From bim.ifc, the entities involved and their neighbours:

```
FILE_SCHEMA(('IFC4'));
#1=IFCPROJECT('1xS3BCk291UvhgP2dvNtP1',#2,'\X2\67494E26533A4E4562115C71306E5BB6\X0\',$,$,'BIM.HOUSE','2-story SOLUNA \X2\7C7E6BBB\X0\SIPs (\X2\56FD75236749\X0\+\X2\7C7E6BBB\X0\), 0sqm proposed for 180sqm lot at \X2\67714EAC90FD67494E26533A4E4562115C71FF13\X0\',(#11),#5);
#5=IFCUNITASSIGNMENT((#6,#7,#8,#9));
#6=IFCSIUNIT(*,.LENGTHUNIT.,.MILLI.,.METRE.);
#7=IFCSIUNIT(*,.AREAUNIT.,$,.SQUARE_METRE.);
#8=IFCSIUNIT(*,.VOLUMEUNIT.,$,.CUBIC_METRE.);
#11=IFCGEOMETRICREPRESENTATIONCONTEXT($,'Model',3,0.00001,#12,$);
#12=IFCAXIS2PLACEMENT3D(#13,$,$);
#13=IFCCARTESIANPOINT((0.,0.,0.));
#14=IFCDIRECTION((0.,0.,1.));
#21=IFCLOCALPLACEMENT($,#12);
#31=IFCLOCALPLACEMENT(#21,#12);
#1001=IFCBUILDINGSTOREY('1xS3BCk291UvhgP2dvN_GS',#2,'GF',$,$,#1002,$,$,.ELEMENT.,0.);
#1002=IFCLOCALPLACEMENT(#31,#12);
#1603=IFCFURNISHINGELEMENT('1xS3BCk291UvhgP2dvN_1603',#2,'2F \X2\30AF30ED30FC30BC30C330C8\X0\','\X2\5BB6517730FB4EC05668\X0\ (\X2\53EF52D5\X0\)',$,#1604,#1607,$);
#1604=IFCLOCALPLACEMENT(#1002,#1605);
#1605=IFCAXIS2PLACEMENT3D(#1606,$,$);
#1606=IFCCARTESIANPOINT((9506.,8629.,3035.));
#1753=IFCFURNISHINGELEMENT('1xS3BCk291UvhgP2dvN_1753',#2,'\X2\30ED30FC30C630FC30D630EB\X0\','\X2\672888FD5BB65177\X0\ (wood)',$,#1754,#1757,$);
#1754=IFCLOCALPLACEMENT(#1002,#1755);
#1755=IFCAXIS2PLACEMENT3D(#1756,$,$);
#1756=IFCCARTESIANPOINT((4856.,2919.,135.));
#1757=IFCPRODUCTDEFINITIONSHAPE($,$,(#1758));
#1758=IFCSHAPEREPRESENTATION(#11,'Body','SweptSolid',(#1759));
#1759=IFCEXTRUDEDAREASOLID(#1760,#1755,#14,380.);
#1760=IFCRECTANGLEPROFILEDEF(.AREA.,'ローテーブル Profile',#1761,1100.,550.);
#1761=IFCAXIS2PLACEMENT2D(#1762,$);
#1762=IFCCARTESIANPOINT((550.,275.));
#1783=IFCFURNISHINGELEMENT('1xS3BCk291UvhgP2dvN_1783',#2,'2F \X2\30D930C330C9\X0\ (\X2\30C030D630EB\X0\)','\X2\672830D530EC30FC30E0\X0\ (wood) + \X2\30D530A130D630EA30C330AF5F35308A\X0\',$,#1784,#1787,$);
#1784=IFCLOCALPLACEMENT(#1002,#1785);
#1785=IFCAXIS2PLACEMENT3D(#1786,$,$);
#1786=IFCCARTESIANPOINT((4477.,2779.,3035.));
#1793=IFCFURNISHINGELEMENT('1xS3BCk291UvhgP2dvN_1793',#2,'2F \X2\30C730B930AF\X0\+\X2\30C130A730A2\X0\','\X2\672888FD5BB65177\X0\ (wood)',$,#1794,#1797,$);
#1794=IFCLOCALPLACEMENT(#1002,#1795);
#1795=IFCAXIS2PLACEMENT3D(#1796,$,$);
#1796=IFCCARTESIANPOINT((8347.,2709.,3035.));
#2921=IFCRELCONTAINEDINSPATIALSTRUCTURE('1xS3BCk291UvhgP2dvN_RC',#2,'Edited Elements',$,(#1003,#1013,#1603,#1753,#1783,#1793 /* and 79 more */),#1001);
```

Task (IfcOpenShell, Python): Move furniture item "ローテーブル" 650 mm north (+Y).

```python
import ifcopenshell
import ifcopenshell.api.geometry
import ifcopenshell.util.placement

model = ifcopenshell.open("bim.ifc")

item = model.by_id(1753)
matrix = ifcopenshell.util.placement.get_local_placement(item.ObjectPlacement)
matrix[1, 3] += 650.0
ifcopenshell.api.geometry.edit_object_placement(model, product=item, matrix=matrix, is_si=False)

print(ifcopenshell.util.placement.get_local_placement(item.ObjectPlacement).round(3) + 0.0)

model.write("bim_updated.ifc")
```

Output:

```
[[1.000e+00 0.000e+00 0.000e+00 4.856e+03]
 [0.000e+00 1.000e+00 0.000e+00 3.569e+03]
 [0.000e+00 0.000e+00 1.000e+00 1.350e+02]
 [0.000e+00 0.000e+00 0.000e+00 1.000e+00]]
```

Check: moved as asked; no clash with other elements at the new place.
